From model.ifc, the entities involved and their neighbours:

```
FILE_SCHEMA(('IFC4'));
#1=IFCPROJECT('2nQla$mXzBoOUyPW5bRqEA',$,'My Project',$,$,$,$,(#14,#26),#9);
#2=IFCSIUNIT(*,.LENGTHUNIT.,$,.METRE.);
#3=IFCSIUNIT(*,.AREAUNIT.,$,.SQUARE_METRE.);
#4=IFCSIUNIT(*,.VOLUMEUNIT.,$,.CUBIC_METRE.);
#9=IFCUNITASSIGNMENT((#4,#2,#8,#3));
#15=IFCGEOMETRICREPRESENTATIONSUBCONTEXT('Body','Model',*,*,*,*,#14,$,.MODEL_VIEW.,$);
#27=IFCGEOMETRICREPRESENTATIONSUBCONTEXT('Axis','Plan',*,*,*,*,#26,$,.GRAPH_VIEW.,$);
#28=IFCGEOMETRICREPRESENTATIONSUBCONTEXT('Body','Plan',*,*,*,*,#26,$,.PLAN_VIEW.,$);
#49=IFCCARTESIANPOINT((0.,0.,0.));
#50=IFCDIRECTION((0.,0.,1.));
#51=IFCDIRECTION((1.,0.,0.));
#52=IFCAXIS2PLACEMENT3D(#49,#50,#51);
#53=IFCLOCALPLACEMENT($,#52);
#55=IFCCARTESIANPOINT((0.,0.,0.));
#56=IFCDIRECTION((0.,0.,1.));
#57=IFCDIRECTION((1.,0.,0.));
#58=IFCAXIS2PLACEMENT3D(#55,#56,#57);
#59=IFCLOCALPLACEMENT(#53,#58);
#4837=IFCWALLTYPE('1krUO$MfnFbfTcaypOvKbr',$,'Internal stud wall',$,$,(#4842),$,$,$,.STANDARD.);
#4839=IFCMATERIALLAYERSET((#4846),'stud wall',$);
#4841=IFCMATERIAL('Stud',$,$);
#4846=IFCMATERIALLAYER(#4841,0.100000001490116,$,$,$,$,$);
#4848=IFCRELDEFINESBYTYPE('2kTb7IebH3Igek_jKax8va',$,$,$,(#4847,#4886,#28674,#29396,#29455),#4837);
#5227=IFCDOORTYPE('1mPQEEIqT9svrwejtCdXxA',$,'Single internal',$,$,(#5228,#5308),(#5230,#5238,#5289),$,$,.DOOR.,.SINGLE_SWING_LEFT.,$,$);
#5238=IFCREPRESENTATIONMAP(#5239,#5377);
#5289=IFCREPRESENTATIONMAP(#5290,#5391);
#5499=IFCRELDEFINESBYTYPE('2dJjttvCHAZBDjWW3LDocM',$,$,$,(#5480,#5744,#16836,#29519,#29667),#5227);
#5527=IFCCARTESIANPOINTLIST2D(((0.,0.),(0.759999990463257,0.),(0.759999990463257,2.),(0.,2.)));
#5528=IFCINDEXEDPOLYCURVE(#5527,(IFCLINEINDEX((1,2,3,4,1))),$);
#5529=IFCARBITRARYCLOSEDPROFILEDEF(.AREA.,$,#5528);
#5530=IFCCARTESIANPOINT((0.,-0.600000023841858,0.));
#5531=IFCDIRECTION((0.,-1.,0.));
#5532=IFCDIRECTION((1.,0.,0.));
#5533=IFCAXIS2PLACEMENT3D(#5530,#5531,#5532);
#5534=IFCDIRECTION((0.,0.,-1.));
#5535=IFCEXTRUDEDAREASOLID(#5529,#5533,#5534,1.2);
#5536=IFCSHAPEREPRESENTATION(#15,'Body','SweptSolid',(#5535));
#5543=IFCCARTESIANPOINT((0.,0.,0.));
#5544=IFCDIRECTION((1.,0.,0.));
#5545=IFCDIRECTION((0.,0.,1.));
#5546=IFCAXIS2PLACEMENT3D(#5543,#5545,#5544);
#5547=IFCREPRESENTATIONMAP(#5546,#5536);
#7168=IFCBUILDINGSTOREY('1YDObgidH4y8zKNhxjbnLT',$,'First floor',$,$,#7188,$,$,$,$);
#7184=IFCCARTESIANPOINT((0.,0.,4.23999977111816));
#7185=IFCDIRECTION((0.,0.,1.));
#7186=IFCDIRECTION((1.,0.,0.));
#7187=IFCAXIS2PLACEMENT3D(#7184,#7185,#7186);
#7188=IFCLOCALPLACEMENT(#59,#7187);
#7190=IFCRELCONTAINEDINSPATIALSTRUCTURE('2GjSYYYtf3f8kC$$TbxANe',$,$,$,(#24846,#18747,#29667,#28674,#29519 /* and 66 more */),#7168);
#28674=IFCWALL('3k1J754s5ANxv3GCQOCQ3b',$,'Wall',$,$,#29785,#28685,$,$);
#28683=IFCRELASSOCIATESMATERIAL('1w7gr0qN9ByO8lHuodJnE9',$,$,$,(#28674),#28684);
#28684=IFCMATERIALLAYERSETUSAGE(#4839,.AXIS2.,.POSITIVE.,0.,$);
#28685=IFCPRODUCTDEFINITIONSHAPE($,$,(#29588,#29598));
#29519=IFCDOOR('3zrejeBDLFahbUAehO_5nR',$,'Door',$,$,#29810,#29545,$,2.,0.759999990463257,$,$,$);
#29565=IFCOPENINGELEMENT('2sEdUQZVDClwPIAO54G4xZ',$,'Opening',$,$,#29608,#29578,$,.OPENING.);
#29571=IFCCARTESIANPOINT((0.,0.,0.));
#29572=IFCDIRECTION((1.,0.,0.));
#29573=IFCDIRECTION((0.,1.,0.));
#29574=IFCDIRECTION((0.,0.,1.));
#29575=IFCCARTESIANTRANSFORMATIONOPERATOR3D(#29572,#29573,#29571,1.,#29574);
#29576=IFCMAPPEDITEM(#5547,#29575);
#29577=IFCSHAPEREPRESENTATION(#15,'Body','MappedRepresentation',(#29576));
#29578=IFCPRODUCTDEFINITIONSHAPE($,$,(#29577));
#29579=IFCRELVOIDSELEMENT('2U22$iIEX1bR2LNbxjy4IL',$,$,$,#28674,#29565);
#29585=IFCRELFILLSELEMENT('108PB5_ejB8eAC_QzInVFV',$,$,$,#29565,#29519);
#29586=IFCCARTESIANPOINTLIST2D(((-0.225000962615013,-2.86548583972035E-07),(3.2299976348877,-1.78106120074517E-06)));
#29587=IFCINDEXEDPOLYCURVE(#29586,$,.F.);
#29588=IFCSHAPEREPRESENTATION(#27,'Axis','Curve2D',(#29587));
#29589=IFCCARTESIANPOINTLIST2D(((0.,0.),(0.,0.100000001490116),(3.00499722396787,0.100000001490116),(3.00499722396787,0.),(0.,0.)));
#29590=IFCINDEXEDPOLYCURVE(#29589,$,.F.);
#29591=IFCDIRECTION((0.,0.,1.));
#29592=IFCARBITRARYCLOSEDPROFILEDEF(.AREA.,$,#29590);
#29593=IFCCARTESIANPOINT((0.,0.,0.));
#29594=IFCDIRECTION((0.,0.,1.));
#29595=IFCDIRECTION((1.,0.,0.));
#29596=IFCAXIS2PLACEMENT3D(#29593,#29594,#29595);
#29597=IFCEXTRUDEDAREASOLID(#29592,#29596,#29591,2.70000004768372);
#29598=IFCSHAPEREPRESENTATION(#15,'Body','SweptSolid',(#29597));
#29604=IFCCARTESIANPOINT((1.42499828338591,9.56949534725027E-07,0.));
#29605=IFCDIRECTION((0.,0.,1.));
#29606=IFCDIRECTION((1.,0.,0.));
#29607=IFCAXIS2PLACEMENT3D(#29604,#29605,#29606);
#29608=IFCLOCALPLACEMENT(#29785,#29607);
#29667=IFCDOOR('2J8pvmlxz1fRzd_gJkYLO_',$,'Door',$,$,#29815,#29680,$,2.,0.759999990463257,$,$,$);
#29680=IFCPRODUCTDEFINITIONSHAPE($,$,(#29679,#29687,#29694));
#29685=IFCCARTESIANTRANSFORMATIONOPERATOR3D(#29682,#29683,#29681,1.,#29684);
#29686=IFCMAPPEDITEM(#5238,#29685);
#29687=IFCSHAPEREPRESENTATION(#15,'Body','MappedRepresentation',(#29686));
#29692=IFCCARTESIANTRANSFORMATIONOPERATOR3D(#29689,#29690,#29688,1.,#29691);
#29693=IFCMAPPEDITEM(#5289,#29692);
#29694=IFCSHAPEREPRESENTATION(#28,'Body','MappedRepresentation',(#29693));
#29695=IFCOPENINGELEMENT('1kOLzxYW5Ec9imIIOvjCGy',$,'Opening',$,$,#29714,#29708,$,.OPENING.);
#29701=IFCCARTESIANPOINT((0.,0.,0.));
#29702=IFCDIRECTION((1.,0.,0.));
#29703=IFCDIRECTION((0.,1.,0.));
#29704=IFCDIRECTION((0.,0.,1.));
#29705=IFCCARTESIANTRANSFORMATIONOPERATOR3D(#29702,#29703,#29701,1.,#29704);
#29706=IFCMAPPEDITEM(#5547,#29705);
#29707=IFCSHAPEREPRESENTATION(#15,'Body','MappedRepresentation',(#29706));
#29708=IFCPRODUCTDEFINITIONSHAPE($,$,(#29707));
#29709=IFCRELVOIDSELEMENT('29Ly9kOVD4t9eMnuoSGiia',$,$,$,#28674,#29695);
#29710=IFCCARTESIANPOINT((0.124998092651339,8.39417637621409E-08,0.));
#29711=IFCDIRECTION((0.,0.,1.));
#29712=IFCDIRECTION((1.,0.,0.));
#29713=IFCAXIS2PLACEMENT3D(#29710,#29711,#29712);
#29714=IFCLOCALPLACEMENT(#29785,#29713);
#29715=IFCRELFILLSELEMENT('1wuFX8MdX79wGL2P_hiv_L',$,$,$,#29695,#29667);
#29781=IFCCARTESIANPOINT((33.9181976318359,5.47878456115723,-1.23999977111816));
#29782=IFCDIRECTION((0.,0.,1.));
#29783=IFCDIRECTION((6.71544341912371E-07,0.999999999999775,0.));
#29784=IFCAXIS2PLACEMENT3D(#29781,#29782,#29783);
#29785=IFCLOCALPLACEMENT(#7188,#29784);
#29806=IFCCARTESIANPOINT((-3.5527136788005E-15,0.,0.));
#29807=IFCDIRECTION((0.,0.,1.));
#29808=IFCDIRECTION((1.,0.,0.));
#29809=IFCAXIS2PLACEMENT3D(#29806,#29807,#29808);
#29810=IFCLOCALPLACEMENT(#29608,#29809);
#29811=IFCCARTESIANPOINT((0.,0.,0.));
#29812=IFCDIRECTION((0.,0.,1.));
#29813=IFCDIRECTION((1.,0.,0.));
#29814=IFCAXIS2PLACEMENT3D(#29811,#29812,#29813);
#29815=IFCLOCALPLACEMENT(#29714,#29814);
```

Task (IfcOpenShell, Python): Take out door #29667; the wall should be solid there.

```python
import ifcopenshell
import ifcopenshell.api.feature
import ifcopenshell.api.root
import ifcopenshell.geom
import ifcopenshell.util.shape

model = ifcopenshell.open("model.ifc")
settings = ifcopenshell.geom.settings()


def volume(element):
    """Net volume in cubic metres, openings subtracted."""
    shape = ifcopenshell.geom.create_shape(settings, element)
    return ifcopenshell.util.shape.get_volume(shape.geometry)


door = model.by_guid("2J8pvmlxz1fRzd_gJkYLO_")
opening = door.FillsVoids[0].RelatingOpeningElement
wall = opening.VoidsElements[0].RelatingBuildingElement
before = volume(wall)

ifcopenshell.api.root.remove_product(model, product=door)
ifcopenshell.api.feature.remove_feature(model, feature=opening)

after = volume(wall)

print(f"wall volume {before:.3f} -> {after:.3f} m3")

model.write("model-out.ifc")
```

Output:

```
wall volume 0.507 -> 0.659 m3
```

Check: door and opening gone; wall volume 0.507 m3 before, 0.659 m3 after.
